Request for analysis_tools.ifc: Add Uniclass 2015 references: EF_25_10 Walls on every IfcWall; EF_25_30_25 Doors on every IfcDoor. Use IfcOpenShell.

First a look at what the model holds.

```python
import ifcopenshell

model = ifcopenshell.open("analysis_tools.ifc")
print(model.schema)
print("classifications:", [c.Name for c in model.by_type("IfcClassification")])
for ifc_class in ("IfcDoor", "IfcRoof", "IfcStair", "IfcWall", "IfcWindow"):
    print(ifc_class, len(model.by_type(ifc_class)))
```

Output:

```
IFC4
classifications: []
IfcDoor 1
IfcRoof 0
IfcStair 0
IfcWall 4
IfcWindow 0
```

```python
import ifcopenshell
import ifcopenshell.api.classification

model = ifcopenshell.open("analysis_tools.ifc")

system = ifcopenshell.api.classification.add_classification(model, classification="Uniclass 2015")

codes = {
    "IfcWall": ("EF_25_10", "Walls"),
    "IfcDoor": ("EF_25_30_25", "Doors"),
}
for ifc_class, (code, name) in codes.items():
    products = model.by_type(ifc_class)
    ifcopenshell.api.classification.add_reference(
        model, products=products, classification=system, identification=code, name=name
    )
    print(code, len(products))

model.write("analysis_tools_edited.ifc")
```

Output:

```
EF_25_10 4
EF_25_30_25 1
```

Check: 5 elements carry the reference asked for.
